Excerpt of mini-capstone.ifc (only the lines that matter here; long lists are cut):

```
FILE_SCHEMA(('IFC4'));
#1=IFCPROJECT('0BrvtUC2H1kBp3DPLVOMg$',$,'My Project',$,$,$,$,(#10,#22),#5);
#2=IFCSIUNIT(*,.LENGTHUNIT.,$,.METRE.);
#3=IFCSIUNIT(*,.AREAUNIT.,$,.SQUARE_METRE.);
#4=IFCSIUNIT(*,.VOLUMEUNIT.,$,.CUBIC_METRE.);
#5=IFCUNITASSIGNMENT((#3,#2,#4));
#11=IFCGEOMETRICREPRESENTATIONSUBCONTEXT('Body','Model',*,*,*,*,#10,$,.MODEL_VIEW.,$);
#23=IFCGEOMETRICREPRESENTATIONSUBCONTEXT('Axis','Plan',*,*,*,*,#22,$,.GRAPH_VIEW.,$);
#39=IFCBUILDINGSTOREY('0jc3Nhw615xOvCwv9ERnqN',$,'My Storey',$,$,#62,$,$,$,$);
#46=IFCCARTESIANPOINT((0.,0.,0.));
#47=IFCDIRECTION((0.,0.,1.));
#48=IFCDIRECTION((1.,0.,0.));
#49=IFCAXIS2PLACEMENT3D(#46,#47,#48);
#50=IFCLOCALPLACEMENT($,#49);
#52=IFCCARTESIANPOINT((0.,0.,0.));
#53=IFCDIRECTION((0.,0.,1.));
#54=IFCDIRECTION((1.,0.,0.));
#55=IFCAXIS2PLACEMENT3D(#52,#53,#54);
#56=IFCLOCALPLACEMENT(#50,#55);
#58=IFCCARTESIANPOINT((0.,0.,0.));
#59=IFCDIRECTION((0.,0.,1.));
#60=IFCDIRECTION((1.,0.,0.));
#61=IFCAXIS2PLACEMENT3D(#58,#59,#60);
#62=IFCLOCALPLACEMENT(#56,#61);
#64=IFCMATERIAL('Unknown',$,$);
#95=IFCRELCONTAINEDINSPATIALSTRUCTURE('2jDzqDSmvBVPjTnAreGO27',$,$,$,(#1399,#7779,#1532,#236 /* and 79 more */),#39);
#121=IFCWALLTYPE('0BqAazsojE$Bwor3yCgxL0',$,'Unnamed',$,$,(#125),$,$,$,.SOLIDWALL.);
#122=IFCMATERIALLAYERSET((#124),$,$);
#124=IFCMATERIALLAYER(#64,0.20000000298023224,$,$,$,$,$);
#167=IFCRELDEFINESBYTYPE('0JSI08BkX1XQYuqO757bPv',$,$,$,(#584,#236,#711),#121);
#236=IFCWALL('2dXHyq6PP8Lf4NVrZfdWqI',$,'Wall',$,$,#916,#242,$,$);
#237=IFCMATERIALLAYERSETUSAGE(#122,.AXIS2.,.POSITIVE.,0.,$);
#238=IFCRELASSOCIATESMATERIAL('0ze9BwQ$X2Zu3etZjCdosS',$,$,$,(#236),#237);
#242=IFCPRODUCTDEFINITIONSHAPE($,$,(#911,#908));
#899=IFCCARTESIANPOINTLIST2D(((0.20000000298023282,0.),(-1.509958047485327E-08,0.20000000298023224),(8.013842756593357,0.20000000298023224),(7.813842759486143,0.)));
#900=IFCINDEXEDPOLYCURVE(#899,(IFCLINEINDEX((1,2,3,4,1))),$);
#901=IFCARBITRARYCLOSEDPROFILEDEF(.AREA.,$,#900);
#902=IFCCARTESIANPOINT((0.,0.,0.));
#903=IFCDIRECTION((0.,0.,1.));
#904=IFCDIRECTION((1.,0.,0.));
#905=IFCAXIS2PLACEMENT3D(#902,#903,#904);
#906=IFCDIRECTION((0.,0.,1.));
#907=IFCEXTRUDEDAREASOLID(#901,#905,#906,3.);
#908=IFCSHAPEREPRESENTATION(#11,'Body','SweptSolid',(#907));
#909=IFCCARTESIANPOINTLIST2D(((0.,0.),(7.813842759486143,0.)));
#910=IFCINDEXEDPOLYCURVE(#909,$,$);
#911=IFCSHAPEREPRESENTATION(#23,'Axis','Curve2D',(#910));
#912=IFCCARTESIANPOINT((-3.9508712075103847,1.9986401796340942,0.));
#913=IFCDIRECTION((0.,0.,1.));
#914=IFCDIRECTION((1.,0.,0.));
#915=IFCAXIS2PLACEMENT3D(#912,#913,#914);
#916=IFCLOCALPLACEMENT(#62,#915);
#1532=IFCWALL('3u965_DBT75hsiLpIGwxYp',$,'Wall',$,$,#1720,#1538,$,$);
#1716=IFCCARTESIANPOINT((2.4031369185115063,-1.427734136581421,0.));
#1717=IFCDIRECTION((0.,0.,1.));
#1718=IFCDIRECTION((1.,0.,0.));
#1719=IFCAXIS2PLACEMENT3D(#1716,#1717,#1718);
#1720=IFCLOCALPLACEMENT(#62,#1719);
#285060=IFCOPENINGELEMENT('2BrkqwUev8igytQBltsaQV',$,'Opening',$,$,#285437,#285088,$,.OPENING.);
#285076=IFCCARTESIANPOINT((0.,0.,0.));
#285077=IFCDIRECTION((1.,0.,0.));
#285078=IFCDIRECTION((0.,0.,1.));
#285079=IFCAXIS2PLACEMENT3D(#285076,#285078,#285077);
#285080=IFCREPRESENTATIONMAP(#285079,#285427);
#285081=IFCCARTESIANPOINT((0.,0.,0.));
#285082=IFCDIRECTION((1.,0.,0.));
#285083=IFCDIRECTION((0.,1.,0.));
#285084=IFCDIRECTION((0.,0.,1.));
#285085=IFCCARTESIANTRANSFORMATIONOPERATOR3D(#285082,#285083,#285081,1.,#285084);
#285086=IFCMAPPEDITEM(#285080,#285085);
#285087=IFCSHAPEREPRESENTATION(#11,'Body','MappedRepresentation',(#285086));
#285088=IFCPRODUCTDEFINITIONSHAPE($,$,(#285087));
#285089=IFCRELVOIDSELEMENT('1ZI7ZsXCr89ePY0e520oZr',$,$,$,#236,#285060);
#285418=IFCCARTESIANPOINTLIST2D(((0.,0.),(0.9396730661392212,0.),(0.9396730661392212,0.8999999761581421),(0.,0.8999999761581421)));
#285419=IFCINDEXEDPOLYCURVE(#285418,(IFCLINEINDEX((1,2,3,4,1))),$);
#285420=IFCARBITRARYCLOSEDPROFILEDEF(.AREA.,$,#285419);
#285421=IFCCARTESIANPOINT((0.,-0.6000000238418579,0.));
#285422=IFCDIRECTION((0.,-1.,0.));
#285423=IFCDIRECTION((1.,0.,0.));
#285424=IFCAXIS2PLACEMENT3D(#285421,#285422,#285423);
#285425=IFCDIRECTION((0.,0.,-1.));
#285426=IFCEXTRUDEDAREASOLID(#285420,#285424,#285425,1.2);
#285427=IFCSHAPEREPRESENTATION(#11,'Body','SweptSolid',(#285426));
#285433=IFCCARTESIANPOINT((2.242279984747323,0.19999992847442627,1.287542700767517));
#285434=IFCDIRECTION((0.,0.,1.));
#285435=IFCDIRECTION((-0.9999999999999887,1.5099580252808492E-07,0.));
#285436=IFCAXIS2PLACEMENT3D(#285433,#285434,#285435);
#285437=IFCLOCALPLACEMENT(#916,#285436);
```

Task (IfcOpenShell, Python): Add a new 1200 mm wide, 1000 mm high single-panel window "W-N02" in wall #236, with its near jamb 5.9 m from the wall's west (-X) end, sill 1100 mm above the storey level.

```python
import numpy as np
import ifcopenshell
import ifcopenshell.api.feature
import ifcopenshell.api.geometry
import ifcopenshell.api.root
import ifcopenshell.api.spatial
import ifcopenshell.geom
import ifcopenshell.util.element
import ifcopenshell.util.placement
import ifcopenshell.util.representation
import ifcopenshell.util.shape
import ifcopenshell.util.unit

model = ifcopenshell.open("mini-capstone.ifc")
unit_scale = ifcopenshell.util.unit.calculate_unit_scale(model)
settings = ifcopenshell.geom.settings()


def volume(element):
    """Net volume in cubic metres, openings subtracted."""
    shape = ifcopenshell.geom.create_shape(settings, element)
    return ifcopenshell.util.shape.get_volume(shape.geometry)


wall = model.by_guid("2dXHyq6PP8Lf4NVrZfdWqI")
storey = ifcopenshell.util.element.get_container(wall, ifc_class="IfcBuildingStorey")
context = ifcopenshell.util.representation.get_context(model, "Model", "Body", "MODEL_VIEW")
before = volume(wall)

width, height, from_end, sill = 1.2, 1, 5.9, 1.1  # metres

# The wall runs along its own X axis, and the end named is its -X end.
wall_shape = ifcopenshell.geom.create_shape(settings, wall)
x, y, z = ifcopenshell.util.shape.get_vertices(wall_shape.geometry).T
start = x.min() + from_end
face, thickness = float(y.min()), float(y.max() - y.min())
wall_matrix = ifcopenshell.util.placement.get_local_placement(wall.ObjectPlacement)
level = ifcopenshell.util.placement.get_local_placement(storey.ObjectPlacement)[2, 3]


def in_wall(x, y):
    """Placement at x, y metres in the wall's axes, at sill height."""
    matrix = wall_matrix.copy()
    matrix[:, 3] = wall_matrix @ np.array([x / unit_scale, y / unit_scale, 0.0, 1.0])
    matrix[2, 3] = level + sill / unit_scale
    return matrix


# Opening: a box that overshoots both wall faces by 50 mm.
opening = ifcopenshell.api.root.create_entity(model, ifc_class="IfcOpeningElement", predefined_type="OPENING")
box = ifcopenshell.api.geometry.add_wall_representation(
    model, context=context, length=width, height=height, thickness=thickness + 0.1
)
ifcopenshell.api.geometry.assign_representation(model, product=opening, representation=box)
ifcopenshell.api.geometry.edit_object_placement(model, product=opening, matrix=in_wall(start, face - 0.05), is_si=False)
ifcopenshell.api.feature.add_feature(model, feature=opening, element=wall)

window = ifcopenshell.api.root.create_entity(model, ifc_class="IfcWindow", name="W-N02", predefined_type="WINDOW")
window.OverallWidth, window.OverallHeight = width / unit_scale, height / unit_scale
window.PartitioningType = "SINGLE_PANEL"
body = ifcopenshell.api.geometry.add_window_representation(
    model,
    context=context,
    overall_width=window.OverallWidth,
    overall_height=window.OverallHeight,
    partition_type="SINGLE_PANEL",
)
ifcopenshell.api.geometry.assign_representation(model, product=window, representation=body)
ifcopenshell.api.spatial.assign_container(model, products=[window], relating_structure=storey)
ifcopenshell.api.feature.add_filling(model, opening=opening, element=window)

# Centre the window in the wall's thickness.
ifcopenshell.api.geometry.edit_object_placement(model, product=window, matrix=in_wall(start, face), is_si=False)
window_shape = ifcopenshell.geom.create_shape(settings, window)
depth = ifcopenshell.util.shape.get_vertices(window_shape.geometry)[:, 1]
offset = face + thickness / 2 - (depth.min() + depth.max()) / 2
ifcopenshell.api.geometry.edit_object_placement(model, product=window, matrix=in_wall(start, offset), is_si=False)

after = volume(wall)

print(f"wall volume {before:.3f} -> {after:.3f} m3")

model.write("mini-capstone_updated.ifc")
```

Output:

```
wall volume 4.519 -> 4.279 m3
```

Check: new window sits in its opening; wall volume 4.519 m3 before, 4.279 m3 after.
